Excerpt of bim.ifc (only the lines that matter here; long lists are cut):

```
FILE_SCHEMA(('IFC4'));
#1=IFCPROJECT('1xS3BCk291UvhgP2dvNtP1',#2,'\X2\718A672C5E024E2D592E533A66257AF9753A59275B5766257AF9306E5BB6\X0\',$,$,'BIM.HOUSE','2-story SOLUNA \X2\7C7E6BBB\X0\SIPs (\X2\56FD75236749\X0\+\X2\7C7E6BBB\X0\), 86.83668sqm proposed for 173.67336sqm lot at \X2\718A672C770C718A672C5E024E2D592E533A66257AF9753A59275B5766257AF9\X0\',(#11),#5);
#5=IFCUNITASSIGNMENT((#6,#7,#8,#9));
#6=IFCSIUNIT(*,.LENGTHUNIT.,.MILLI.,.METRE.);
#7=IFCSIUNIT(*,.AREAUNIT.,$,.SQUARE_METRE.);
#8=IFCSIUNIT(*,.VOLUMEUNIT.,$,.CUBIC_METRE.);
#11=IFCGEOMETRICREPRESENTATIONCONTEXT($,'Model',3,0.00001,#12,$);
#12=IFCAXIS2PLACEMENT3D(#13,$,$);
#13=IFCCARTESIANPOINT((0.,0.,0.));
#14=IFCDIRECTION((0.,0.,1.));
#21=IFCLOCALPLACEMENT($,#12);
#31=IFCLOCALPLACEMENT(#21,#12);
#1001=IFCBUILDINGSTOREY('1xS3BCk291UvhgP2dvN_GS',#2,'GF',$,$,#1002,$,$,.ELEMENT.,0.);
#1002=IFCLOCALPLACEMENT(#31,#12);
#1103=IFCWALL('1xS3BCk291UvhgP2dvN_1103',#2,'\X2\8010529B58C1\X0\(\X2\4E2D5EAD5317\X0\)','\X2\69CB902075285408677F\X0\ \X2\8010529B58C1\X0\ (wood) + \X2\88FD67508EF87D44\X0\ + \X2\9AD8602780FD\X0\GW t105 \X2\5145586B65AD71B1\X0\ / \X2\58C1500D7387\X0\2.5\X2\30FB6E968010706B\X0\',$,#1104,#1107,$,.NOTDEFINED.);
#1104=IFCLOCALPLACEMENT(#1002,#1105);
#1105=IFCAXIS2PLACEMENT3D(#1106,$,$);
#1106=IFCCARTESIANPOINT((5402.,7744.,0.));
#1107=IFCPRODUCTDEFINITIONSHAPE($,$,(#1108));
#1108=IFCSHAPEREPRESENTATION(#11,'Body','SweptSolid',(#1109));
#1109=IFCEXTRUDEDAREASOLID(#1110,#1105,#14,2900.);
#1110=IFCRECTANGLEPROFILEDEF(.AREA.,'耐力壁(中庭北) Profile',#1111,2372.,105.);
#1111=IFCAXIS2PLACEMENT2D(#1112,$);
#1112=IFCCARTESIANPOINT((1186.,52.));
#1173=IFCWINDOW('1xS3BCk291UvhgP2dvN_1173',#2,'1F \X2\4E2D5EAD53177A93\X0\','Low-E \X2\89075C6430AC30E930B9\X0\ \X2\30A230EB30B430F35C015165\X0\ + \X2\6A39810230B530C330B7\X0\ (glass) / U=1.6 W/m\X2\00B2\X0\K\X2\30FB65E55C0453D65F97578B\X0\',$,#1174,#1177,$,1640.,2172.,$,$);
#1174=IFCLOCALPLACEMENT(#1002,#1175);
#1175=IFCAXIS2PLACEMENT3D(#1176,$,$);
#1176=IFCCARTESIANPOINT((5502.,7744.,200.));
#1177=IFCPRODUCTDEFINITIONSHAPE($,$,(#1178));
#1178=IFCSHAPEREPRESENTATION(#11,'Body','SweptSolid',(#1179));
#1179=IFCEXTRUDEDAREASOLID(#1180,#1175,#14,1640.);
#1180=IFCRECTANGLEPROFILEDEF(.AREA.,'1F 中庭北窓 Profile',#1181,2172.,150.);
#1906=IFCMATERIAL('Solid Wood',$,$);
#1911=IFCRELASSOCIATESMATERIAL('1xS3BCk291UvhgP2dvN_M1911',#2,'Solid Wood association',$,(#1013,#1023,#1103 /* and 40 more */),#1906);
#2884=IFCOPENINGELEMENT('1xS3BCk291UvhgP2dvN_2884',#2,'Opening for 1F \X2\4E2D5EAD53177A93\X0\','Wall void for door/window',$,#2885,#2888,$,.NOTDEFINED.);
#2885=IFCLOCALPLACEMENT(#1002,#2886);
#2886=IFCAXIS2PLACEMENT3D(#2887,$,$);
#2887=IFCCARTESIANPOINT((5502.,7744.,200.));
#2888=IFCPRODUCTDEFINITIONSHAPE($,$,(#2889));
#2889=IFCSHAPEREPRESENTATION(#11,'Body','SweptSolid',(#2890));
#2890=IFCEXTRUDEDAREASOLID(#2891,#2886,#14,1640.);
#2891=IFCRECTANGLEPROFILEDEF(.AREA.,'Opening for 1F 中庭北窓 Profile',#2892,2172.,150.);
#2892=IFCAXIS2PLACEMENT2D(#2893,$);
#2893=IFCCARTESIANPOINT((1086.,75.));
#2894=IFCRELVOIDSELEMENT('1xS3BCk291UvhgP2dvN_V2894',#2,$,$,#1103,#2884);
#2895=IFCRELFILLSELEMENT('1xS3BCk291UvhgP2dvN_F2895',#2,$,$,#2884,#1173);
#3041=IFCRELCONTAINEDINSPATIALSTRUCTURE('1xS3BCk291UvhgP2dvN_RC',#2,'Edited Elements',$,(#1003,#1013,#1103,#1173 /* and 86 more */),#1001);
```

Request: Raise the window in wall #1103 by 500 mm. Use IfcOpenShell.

```python
import numpy as np
import ifcopenshell
import ifcopenshell.api.geometry
import ifcopenshell.util.placement
import ifcopenshell.util.unit

model = ifcopenshell.open("bim.ifc")
unit_scale = ifcopenshell.util.unit.calculate_unit_scale(model)

window = model.by_id(1173)
opening = window.FillsVoids[0].RelatingOpeningElement
dz = 500.0

shift = np.array([0.0, 0.0, dz])
# The window is not placed relative to its opening, so move both.
for product in (opening, window):
    matrix = ifcopenshell.util.placement.get_local_placement(product.ObjectPlacement)
    matrix[:3, 3] += shift
    ifcopenshell.api.geometry.edit_object_placement(model, product=product, matrix=matrix, is_si=False)

print(f"moved by {dz * unit_scale:+.3f} m")

model.write("bim-out.ifc")
```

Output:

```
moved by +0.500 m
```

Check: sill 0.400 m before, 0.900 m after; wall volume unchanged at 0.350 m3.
